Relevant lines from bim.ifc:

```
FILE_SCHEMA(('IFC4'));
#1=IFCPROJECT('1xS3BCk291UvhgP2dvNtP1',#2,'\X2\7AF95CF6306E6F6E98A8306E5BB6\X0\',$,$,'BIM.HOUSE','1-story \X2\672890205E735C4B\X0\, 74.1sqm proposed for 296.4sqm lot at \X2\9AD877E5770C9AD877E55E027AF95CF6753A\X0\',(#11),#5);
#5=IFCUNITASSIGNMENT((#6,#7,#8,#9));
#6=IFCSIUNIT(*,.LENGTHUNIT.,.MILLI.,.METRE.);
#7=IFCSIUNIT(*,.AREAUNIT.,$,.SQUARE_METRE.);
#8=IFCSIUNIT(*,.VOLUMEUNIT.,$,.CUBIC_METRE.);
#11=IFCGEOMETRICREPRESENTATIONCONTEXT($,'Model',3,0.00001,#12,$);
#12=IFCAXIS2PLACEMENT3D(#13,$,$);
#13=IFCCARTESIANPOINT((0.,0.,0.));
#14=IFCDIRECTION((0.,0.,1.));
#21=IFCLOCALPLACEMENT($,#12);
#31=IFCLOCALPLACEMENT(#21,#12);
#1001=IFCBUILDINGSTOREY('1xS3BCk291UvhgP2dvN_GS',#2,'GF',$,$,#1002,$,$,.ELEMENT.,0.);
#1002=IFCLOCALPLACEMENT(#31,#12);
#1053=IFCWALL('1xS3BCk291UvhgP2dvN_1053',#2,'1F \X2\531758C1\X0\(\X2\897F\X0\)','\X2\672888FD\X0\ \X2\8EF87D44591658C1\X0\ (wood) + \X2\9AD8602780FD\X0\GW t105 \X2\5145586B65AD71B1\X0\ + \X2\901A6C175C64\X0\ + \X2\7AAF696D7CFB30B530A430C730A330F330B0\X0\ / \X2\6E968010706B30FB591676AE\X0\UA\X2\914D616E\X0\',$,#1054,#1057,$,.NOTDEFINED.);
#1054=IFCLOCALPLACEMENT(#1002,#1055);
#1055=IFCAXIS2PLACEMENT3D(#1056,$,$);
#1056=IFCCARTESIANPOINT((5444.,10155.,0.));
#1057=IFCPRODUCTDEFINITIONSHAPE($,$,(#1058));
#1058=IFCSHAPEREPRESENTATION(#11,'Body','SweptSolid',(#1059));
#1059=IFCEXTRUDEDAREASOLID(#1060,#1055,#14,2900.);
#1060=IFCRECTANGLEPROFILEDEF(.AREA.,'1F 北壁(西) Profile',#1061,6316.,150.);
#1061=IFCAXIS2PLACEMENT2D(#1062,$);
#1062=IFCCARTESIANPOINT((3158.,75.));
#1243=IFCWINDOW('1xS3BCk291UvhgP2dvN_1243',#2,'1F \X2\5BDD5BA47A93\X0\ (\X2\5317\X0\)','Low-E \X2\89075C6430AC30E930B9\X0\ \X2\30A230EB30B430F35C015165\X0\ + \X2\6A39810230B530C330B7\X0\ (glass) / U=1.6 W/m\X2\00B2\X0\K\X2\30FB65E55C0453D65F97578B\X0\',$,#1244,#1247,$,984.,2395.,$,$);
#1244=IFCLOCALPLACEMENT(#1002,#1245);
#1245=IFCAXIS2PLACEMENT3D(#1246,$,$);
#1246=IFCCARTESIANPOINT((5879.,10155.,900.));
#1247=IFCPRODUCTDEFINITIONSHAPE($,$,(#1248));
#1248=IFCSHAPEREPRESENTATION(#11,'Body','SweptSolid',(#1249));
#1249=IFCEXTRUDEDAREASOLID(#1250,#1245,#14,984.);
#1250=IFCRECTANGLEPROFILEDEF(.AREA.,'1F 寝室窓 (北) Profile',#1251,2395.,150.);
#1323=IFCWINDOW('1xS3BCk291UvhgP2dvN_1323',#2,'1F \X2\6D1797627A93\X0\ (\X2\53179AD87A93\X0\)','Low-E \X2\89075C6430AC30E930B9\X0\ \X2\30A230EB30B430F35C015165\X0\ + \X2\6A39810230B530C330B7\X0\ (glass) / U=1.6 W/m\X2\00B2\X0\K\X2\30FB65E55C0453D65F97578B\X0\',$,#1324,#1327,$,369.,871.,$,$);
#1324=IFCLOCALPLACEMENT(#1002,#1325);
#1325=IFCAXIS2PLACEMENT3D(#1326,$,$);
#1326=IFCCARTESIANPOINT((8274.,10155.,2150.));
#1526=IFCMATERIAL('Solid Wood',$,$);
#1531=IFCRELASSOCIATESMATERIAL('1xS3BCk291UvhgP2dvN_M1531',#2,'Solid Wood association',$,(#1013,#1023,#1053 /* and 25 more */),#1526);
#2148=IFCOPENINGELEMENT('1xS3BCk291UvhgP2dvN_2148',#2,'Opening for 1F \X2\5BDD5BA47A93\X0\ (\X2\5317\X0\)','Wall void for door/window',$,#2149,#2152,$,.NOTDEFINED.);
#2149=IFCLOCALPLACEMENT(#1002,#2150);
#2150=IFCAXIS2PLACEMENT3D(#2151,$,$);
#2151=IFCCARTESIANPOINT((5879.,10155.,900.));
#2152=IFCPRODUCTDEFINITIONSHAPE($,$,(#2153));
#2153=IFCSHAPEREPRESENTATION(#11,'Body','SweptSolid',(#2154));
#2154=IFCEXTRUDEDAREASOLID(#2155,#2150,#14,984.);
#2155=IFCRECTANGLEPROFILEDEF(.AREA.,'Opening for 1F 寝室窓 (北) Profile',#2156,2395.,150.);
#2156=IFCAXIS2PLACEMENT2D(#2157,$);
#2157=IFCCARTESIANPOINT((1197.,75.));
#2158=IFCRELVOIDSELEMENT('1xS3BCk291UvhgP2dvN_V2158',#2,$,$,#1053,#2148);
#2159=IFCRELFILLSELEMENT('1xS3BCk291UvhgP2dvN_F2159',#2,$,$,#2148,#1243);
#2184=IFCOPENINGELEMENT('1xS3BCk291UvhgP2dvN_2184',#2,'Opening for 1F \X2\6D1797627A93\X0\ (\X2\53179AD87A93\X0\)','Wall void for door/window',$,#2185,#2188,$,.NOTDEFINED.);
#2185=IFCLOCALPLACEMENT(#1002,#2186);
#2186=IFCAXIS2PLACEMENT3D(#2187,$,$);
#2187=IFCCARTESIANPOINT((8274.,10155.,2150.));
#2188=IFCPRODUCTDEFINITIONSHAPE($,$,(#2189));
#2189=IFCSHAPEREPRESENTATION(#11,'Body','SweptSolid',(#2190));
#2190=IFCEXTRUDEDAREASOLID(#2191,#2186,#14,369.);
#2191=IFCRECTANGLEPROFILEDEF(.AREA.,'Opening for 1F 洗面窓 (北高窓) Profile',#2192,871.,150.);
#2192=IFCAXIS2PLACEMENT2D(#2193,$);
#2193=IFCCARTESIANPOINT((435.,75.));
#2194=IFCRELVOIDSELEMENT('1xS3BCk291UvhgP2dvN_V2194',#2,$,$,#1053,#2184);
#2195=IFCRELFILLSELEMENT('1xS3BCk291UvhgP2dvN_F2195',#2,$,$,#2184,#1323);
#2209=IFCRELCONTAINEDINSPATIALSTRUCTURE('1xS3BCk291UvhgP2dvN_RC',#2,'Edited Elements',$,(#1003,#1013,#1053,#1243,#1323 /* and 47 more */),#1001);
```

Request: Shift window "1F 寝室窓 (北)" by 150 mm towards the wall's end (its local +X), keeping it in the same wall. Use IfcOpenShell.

```python
import ifcopenshell
import ifcopenshell.api.geometry
import ifcopenshell.util.placement

model = ifcopenshell.open("bim.ifc")

window = model.by_guid("1xS3BCk291UvhgP2dvN_1243")
opening = window.FillsVoids[0].RelatingOpeningElement
wall = opening.VoidsElements[0].RelatingBuildingElement

wall_matrix = ifcopenshell.util.placement.get_local_placement(wall.ObjectPlacement)
shift = wall_matrix[:3, 0] * 150.0
before = ifcopenshell.util.placement.get_local_placement(window.ObjectPlacement)[:3, 3].copy()

# The window is not placed relative to its opening, so move both.
for product in (opening, window):
    matrix = ifcopenshell.util.placement.get_local_placement(product.ObjectPlacement)
    matrix[:3, 3] += shift
    ifcopenshell.api.geometry.edit_object_placement(model, product=product, matrix=matrix, is_si=False)

after = ifcopenshell.util.placement.get_local_placement(window.ObjectPlacement)[:3, 3]
print("window moved by", (after - before).round(3) + 0.0)

model.write("bim_edited.ifc")
```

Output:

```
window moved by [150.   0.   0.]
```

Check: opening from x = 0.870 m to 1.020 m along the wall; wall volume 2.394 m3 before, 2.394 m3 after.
